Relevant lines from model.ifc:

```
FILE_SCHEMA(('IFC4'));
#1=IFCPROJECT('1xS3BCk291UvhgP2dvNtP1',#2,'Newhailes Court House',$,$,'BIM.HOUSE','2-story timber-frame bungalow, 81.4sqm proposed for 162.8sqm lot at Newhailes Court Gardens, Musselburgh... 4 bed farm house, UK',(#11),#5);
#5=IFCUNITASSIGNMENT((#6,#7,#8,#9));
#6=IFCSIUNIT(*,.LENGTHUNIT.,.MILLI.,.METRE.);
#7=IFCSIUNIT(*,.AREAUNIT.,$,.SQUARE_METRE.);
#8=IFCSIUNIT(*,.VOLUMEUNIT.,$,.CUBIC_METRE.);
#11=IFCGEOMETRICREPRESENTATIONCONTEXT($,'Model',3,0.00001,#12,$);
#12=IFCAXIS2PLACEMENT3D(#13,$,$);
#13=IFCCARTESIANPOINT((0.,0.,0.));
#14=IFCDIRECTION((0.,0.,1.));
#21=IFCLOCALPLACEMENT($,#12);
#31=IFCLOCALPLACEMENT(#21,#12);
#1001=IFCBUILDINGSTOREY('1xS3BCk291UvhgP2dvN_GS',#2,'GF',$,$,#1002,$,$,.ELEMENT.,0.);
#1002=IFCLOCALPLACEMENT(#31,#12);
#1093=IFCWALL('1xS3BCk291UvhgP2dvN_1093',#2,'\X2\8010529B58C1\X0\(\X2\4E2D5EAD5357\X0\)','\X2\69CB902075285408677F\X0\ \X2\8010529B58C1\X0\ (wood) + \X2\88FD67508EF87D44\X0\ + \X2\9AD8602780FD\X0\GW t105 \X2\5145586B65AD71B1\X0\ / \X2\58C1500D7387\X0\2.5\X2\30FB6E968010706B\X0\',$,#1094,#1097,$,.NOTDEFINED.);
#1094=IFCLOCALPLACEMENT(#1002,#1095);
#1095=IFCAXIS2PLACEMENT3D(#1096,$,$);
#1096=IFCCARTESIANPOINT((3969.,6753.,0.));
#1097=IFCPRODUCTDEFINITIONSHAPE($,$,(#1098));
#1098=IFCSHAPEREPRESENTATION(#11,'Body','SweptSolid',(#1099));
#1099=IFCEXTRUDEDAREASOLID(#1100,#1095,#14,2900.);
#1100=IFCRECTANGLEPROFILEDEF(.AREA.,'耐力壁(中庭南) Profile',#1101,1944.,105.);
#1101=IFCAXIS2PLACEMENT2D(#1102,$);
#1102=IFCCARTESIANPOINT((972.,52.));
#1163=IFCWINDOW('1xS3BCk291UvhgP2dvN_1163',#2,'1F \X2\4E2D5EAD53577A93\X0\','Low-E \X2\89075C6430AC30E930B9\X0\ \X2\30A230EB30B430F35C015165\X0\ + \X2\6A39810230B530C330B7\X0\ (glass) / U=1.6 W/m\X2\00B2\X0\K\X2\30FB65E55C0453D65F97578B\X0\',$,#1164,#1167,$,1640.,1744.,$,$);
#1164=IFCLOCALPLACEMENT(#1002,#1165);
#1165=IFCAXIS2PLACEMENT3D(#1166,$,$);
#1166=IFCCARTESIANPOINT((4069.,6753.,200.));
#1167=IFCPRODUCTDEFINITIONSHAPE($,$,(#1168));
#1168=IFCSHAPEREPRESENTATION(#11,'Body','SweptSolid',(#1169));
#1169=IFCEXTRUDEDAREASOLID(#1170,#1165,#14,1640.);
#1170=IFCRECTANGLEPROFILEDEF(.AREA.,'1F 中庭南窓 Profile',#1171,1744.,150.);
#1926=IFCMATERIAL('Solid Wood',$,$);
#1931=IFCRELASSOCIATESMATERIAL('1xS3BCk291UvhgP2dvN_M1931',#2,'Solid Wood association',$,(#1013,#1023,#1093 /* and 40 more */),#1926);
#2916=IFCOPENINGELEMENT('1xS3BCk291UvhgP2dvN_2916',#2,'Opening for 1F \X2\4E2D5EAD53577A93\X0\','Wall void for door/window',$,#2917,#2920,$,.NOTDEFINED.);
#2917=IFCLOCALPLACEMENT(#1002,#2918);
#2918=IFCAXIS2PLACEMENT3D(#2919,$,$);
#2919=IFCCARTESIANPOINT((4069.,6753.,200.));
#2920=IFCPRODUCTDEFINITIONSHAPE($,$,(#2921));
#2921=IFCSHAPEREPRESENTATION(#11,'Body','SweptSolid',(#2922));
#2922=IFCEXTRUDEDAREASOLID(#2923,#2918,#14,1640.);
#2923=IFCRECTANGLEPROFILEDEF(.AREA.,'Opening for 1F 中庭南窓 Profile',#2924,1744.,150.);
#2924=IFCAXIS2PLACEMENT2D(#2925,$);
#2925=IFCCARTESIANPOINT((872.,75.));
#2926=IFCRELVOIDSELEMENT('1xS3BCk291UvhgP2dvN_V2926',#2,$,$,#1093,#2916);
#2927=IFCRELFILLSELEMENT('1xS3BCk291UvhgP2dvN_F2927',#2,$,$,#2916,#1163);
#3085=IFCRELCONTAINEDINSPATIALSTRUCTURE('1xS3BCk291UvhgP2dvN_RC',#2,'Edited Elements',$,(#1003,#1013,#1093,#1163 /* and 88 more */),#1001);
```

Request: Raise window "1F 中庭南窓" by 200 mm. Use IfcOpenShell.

```python
import numpy as np
import ifcopenshell
import ifcopenshell.api.geometry
import ifcopenshell.util.placement
import ifcopenshell.util.unit

model = ifcopenshell.open("model.ifc")
unit_scale = ifcopenshell.util.unit.calculate_unit_scale(model)

window = model.by_guid("1xS3BCk291UvhgP2dvN_1163")
opening = window.FillsVoids[0].RelatingOpeningElement
dz = 200.0

shift = np.array([0.0, 0.0, dz])
# The window is not placed relative to its opening, so move both.
for product in (opening, window):
    matrix = ifcopenshell.util.placement.get_local_placement(product.ObjectPlacement)
    matrix[:3, 3] += shift
    ifcopenshell.api.geometry.edit_object_placement(model, product=product, matrix=matrix, is_si=False)

print(f"moved by {dz * unit_scale:+.3f} m")

model.write("model_updated.ifc")
```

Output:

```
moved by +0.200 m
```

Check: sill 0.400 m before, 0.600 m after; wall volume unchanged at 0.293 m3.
